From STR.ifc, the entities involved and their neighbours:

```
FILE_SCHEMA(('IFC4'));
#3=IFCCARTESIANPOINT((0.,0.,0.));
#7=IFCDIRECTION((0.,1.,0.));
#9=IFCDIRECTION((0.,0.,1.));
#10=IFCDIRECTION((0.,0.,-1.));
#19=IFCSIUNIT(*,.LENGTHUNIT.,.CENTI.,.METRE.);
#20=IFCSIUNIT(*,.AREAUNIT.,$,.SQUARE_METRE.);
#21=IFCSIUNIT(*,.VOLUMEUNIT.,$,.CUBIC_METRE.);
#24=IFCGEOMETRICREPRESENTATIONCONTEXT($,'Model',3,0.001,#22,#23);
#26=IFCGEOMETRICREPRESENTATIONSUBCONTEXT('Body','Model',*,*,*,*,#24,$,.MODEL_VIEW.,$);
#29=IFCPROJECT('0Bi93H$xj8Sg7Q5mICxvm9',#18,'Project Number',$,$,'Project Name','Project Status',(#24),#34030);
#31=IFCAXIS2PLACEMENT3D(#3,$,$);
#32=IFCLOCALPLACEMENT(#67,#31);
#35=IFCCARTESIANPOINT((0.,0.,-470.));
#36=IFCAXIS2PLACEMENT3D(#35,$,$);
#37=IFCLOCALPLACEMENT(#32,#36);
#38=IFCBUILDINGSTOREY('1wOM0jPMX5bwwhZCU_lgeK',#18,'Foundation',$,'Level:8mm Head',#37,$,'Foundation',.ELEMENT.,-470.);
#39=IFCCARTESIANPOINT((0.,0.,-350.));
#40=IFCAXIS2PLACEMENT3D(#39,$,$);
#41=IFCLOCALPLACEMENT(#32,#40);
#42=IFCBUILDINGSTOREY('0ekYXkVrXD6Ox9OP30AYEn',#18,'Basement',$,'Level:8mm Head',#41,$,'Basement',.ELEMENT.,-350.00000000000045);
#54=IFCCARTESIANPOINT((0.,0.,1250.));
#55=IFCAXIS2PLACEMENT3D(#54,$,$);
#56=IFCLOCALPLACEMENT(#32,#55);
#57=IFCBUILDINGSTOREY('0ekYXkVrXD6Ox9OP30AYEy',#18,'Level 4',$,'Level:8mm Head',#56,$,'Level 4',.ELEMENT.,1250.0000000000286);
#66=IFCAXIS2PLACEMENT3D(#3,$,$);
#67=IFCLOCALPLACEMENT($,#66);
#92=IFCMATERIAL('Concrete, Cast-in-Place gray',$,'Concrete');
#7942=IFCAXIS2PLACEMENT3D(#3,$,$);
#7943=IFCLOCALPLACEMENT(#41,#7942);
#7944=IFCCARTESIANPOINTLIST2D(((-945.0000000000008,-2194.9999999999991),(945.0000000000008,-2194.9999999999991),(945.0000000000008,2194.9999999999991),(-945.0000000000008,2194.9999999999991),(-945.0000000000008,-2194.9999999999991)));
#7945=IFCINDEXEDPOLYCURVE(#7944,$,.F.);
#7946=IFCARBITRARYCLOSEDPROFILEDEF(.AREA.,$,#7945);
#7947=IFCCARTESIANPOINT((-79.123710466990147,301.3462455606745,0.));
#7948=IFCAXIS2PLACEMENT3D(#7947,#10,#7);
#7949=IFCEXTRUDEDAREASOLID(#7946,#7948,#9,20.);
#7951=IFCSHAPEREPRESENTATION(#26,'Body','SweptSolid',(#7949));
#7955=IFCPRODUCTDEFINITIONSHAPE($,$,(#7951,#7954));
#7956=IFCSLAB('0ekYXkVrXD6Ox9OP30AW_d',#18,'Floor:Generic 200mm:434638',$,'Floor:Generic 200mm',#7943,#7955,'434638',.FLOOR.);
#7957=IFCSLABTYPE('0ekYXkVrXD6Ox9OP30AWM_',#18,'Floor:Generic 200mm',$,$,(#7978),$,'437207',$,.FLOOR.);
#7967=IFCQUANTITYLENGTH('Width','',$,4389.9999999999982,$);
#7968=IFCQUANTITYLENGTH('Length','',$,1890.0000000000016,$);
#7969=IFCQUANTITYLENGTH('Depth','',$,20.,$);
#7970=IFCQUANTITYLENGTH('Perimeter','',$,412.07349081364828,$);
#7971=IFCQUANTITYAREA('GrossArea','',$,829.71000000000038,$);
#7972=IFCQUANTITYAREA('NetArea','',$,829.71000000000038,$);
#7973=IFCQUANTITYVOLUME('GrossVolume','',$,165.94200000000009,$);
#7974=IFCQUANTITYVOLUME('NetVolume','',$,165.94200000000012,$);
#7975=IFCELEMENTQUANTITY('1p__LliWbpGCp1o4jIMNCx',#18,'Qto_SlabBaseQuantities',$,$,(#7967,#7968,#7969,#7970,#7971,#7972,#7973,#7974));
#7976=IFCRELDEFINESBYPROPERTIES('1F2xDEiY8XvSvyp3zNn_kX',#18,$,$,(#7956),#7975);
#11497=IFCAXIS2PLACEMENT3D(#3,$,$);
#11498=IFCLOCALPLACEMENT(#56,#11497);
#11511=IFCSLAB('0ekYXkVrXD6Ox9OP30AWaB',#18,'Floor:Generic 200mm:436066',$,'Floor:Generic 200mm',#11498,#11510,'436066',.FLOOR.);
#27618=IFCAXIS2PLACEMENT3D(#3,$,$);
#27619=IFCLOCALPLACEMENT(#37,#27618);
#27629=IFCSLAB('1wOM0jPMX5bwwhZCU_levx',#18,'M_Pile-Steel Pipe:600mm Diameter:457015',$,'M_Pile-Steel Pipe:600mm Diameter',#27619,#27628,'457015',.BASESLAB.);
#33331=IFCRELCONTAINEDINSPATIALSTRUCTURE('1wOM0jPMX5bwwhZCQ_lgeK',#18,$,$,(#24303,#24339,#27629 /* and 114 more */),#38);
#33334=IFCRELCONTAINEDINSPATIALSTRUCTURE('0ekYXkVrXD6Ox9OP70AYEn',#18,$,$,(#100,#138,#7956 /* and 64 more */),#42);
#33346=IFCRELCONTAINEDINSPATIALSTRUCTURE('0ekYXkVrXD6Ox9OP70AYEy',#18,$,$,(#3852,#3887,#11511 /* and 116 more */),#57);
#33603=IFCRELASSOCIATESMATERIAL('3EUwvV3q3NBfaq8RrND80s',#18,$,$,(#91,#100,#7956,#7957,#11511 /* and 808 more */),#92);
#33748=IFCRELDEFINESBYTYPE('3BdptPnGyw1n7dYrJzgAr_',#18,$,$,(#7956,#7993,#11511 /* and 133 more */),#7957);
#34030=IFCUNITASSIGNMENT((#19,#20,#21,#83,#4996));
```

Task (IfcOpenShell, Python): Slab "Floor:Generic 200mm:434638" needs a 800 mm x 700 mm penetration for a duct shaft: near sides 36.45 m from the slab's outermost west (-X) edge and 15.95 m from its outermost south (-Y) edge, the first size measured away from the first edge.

```python
import numpy as np
import ifcopenshell
import ifcopenshell.api.feature
import ifcopenshell.api.geometry
import ifcopenshell.api.pset
import ifcopenshell.api.root
import ifcopenshell.geom
import ifcopenshell.util.element
import ifcopenshell.util.placement
import ifcopenshell.util.representation
import ifcopenshell.util.shape
import ifcopenshell.util.unit

model = ifcopenshell.open("STR.ifc")
unit_scale = ifcopenshell.util.unit.calculate_unit_scale(model)
area_scale = ifcopenshell.util.unit.calculate_unit_scale(model, "AREAUNIT")
volume_scale = ifcopenshell.util.unit.calculate_unit_scale(model, "VOLUMEUNIT")
settings = ifcopenshell.geom.settings()


def volume(element):
    """Net volume in cubic metres, openings subtracted."""
    shape = ifcopenshell.geom.create_shape(settings, element)
    return ifcopenshell.util.shape.get_volume(shape.geometry)


slab = model.by_id(7956)
before = volume(slab)

# Extent in the slab's own axes, in metres. The edges named are its -X and -Y sides.
slab_shape = ifcopenshell.geom.create_shape(settings, slab)
vertices = ifcopenshell.util.shape.get_vertices(slab_shape.geometry)
x_min, y_min, bottom = vertices.min(axis=0)
top = vertices[:, 2].max()

opening = ifcopenshell.api.root.create_entity(model, ifc_class="IfcOpeningElement", name="Duct shaft opening", predefined_type="OPENING")
context = ifcopenshell.util.representation.get_context(model, "Model", "Body", "MODEL_VIEW")
width, depth = 0.8, 0.7
outline = [(0.0, 0.0), (width, 0.0), (width, depth), (0.0, depth), (0.0, 0.0)]
# Overshoot both faces by 50 mm so the cut is clean.
shape = ifcopenshell.api.geometry.add_slab_representation(
    model, context=context, depth=top - bottom + 0.1, polyline=outline
)
ifcopenshell.api.geometry.assign_representation(model, product=opening, representation=shape)

matrix = ifcopenshell.util.placement.get_local_placement(slab.ObjectPlacement)
matrix[:, 3] = matrix @ np.append(np.array([x_min + 36.45, y_min + 15.95, bottom - 0.05]) / unit_scale, 1.0)
ifcopenshell.api.geometry.edit_object_placement(model, product=opening, matrix=matrix, is_si=False)
ifcopenshell.api.feature.add_feature(model, feature=opening, element=slab)

after = volume(slab)

# Update the slab's stored quantities.
qto = model.by_id(ifcopenshell.util.element.get_pset(slab, "Qto_SlabBaseQuantities", should_inherit=False)["id"])
ifcopenshell.api.pset.edit_qto(model, qto=qto, properties={
    "NetArea": after / (top - bottom) / area_scale,
    "NetVolume": after / volume_scale,
})

print(f"slab volume {before:.3f} -> {after:.3f} m3")

model.write("STR_v2.ifc")
```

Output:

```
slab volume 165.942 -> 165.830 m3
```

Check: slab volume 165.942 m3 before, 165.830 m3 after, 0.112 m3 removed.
